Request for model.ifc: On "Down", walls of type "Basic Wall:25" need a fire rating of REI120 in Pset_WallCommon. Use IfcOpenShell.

First a look at what the model holds.

```python
import ifcopenshell
import ifcopenshell.util.element

model = ifcopenshell.open("model.ifc")
print(model.schema)
storey = next(s for s in model.by_type("IfcBuildingStorey") if s.Name == "Down")
walls = [e for e in ifcopenshell.util.element.get_decomposition(storey) if e.is_a("IfcWall")]
seen = {}
for e in walls:
    element_type = ifcopenshell.util.element.get_type(e)
    key = (element_type.Name if element_type != e and element_type else None, ifcopenshell.util.element.get_pset(e, "Pset_WallCommon", "FireRating"))
    seen[key] = seen.get(key, 0) + 1
for (name, value), count in sorted(seen.items(), key=str):
    print(count, "x", name, "|", value)
```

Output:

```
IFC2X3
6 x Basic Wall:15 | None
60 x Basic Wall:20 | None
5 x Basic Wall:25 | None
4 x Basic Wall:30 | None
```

```python
import ifcopenshell
import ifcopenshell.api.pset
import ifcopenshell.util.element

model = ifcopenshell.open("model.ifc")

storey = next(s for s in model.by_type("IfcBuildingStorey") if s.Name == "Down")
walls = [e for e in ifcopenshell.util.element.get_decomposition(storey) if e.is_a("IfcWall")]

count = 0
for e in walls:
    element_type = ifcopenshell.util.element.get_type(e)
    if element_type in (None, e) or element_type.Name != "Basic Wall:25":
        continue
    # add_pset returns the element's existing set when there is one.
    pset = ifcopenshell.api.pset.add_pset(model, product=e, name="Pset_WallCommon")
    ifcopenshell.api.pset.edit_pset(model, pset=pset, properties={"FireRating": "REI120"})
    count += 1

print(count, "walls updated")

model.write("model_updated.ifc")
```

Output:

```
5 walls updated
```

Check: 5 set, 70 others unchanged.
